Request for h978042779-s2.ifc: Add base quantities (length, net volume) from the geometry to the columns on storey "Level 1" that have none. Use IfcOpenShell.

First a look at what the model holds.

```python
import ifcopenshell
import ifcopenshell.util.element
import ifcopenshell.util.unit

model = ifcopenshell.open("h978042779-s2.ifc")
print(model.schema)
for unit_type in ("LENGTHUNIT", "AREAUNIT", "VOLUMEUNIT"):
    print(unit_type, ifcopenshell.util.unit.calculate_unit_scale(model, unit_type))
storey = next(s for s in model.by_type("IfcBuildingStorey") if s.Name == "Level 1")
columns = [e for e in ifcopenshell.util.element.get_decomposition(storey) if e.is_a("IfcColumn")]
for e in sorted(columns, key=lambda e: e.id()):
    print(e.id(), e.is_a(), e.Name, list(ifcopenshell.util.element.get_psets(e, qtos_only=True)), sep=" | ")
```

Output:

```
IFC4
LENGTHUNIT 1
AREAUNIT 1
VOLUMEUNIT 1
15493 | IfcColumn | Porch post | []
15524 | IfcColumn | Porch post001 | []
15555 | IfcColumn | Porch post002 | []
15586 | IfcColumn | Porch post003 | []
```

```python
import ifcopenshell
import ifcopenshell.api.pset
import ifcopenshell.geom
import ifcopenshell.util.element
import ifcopenshell.util.shape
import ifcopenshell.util.unit

model = ifcopenshell.open("h978042779-s2.ifc")
unit_scale = ifcopenshell.util.unit.calculate_unit_scale(model)
volume_scale = ifcopenshell.util.unit.calculate_unit_scale(model, "VOLUMEUNIT")
settings = ifcopenshell.geom.settings()

storey = next(s for s in model.by_type("IfcBuildingStorey") if s.Name == "Level 1")
columns = [e for e in ifcopenshell.util.element.get_decomposition(storey) if e.is_a("IfcColumn")]

for e in sorted(columns, key=lambda e: e.id()):
    if ifcopenshell.util.element.get_psets(e, qtos_only=True, should_inherit=False):
        continue
    # Geometry comes back in metres, in the element's own axes.
    shape = ifcopenshell.geom.create_shape(settings, e)
    values = {
        "Length": ifcopenshell.util.shape.get_z(shape.geometry) / unit_scale,
        "NetVolume": ifcopenshell.util.shape.get_volume(shape.geometry) / volume_scale,
    }
    qto = ifcopenshell.api.pset.add_qto(model, product=e, name="Qto_ColumnBaseQuantities")
    ifcopenshell.api.pset.edit_qto(model, qto=qto, properties=values)
    print(e.id(), {k: round(v, 3) for k, v in values.items()})

model.write("h978042779-s2_rev.ifc")
```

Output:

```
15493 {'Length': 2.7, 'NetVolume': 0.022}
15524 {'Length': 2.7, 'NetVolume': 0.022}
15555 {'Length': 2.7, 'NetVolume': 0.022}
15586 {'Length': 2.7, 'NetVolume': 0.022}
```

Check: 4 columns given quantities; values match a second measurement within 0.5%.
